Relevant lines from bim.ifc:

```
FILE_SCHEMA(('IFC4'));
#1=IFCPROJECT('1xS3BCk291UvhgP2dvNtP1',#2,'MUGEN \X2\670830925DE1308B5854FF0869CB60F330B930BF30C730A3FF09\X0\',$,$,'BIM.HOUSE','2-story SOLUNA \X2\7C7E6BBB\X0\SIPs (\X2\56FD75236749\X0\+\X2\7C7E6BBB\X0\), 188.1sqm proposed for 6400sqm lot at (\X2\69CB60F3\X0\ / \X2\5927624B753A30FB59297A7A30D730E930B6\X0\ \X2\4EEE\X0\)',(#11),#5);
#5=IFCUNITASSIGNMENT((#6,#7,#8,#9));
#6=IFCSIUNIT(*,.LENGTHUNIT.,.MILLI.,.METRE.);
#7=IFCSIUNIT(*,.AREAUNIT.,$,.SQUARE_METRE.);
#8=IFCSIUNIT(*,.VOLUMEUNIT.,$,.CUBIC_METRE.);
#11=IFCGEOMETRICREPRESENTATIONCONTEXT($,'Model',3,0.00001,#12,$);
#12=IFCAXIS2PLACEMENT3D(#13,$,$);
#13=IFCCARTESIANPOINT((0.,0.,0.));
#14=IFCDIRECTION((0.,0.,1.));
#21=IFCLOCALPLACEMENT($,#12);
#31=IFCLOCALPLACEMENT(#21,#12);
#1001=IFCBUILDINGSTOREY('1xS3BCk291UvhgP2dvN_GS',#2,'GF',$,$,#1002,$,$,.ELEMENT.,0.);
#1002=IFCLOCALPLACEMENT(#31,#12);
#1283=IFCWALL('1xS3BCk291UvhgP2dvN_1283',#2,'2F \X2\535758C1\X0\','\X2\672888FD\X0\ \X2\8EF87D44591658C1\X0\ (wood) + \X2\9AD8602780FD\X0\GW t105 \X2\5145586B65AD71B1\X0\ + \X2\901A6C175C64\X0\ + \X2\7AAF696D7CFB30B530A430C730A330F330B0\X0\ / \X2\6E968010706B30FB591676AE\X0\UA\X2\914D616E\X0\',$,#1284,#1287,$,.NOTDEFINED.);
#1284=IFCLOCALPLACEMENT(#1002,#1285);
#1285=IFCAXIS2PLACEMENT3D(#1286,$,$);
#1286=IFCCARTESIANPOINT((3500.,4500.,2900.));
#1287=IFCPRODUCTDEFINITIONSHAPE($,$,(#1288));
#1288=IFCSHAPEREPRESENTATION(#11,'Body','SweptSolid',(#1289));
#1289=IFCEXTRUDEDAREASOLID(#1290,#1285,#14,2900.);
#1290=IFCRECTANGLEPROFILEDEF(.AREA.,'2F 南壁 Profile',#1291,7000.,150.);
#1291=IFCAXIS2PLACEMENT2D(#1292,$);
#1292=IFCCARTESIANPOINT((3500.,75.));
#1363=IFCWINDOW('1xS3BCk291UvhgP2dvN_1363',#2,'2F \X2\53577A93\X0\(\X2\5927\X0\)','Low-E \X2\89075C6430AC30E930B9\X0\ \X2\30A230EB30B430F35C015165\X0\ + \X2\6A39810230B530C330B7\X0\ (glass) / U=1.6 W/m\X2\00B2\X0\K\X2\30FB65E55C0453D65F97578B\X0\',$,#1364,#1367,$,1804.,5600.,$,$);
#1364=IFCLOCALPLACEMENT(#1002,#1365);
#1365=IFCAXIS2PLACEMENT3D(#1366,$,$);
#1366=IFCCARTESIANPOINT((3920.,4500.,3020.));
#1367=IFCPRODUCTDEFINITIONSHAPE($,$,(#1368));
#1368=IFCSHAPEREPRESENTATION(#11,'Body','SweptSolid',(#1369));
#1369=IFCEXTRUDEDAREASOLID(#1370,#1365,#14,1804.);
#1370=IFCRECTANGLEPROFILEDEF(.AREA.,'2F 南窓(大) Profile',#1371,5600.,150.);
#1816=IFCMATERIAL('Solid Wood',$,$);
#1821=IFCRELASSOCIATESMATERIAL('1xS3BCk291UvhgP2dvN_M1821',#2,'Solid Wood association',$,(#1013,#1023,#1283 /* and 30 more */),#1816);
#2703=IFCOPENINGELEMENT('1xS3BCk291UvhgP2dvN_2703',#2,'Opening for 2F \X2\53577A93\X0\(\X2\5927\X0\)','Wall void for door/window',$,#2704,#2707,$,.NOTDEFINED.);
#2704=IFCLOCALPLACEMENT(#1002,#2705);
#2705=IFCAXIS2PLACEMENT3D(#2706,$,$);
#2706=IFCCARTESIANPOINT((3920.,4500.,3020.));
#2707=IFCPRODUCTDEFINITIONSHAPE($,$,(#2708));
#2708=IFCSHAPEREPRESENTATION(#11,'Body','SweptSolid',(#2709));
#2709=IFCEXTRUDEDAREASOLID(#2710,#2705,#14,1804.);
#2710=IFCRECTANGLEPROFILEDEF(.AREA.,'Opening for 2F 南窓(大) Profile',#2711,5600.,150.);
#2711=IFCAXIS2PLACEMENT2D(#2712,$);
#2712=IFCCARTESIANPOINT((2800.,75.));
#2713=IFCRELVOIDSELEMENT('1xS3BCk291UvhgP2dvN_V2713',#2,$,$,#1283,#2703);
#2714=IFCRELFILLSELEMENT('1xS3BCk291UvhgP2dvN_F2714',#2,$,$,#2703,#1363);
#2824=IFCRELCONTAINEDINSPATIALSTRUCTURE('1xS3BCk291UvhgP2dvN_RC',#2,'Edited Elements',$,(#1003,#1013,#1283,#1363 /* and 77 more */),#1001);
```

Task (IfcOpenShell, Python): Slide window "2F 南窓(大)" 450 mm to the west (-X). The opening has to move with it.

```python
import ifcopenshell
import ifcopenshell.api.geometry
import ifcopenshell.util.placement
import ifcopenshell.util.unit

model = ifcopenshell.open("bim.ifc")
unit_scale = ifcopenshell.util.unit.calculate_unit_scale(model)

window = model.by_guid("1xS3BCk291UvhgP2dvN_1363")
opening = window.FillsVoids[0].RelatingOpeningElement
wall = opening.VoidsElements[0].RelatingBuildingElement

wall_matrix = ifcopenshell.util.placement.get_local_placement(wall.ObjectPlacement)
shift = wall_matrix[:3, 0] * -0.45 / unit_scale
before = ifcopenshell.util.placement.get_local_placement(window.ObjectPlacement)[:3, 3].copy()

# The window is not placed relative to its opening, so move both.
for product in (opening, window):
    matrix = ifcopenshell.util.placement.get_local_placement(product.ObjectPlacement)
    matrix[:3, 3] += shift
    ifcopenshell.api.geometry.edit_object_placement(model, product=product, matrix=matrix, is_si=False)

after = ifcopenshell.util.placement.get_local_placement(window.ObjectPlacement)[:3, 3]
print("window moved by", (after - before).round(3) + 0.0)

model.write("bim_edited.ifc")
```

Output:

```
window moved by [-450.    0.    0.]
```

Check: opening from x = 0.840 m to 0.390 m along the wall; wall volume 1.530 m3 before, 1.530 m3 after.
